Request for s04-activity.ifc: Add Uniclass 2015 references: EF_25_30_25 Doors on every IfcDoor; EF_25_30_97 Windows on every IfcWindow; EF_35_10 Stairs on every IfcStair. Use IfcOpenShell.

First a look at what the model holds.

```python
import ifcopenshell

model = ifcopenshell.open("s04-activity.ifc")
print(model.schema)
print("classifications:", [c.Name for c in model.by_type("IfcClassification")])
for ifc_class in ("IfcDoor", "IfcRoof", "IfcStair", "IfcWall", "IfcWindow"):
    print(ifc_class, len(model.by_type(ifc_class)))
```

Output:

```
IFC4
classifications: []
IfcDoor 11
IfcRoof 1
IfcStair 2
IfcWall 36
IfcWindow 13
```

```python
import ifcopenshell
import ifcopenshell.api.classification

model = ifcopenshell.open("s04-activity.ifc")

system = ifcopenshell.api.classification.add_classification(model, classification="Uniclass 2015")

codes = {
    "IfcDoor": ("EF_25_30_25", "Doors"),
    "IfcWindow": ("EF_25_30_97", "Windows"),
    "IfcStair": ("EF_35_10", "Stairs"),
}
for ifc_class, (code, name) in codes.items():
    products = model.by_type(ifc_class)
    ifcopenshell.api.classification.add_reference(
        model, products=products, classification=system, identification=code, name=name
    )
    print(code, len(products))

model.write("s04-activity_updated.ifc")
```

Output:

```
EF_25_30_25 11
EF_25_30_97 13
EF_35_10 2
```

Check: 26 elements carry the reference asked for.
